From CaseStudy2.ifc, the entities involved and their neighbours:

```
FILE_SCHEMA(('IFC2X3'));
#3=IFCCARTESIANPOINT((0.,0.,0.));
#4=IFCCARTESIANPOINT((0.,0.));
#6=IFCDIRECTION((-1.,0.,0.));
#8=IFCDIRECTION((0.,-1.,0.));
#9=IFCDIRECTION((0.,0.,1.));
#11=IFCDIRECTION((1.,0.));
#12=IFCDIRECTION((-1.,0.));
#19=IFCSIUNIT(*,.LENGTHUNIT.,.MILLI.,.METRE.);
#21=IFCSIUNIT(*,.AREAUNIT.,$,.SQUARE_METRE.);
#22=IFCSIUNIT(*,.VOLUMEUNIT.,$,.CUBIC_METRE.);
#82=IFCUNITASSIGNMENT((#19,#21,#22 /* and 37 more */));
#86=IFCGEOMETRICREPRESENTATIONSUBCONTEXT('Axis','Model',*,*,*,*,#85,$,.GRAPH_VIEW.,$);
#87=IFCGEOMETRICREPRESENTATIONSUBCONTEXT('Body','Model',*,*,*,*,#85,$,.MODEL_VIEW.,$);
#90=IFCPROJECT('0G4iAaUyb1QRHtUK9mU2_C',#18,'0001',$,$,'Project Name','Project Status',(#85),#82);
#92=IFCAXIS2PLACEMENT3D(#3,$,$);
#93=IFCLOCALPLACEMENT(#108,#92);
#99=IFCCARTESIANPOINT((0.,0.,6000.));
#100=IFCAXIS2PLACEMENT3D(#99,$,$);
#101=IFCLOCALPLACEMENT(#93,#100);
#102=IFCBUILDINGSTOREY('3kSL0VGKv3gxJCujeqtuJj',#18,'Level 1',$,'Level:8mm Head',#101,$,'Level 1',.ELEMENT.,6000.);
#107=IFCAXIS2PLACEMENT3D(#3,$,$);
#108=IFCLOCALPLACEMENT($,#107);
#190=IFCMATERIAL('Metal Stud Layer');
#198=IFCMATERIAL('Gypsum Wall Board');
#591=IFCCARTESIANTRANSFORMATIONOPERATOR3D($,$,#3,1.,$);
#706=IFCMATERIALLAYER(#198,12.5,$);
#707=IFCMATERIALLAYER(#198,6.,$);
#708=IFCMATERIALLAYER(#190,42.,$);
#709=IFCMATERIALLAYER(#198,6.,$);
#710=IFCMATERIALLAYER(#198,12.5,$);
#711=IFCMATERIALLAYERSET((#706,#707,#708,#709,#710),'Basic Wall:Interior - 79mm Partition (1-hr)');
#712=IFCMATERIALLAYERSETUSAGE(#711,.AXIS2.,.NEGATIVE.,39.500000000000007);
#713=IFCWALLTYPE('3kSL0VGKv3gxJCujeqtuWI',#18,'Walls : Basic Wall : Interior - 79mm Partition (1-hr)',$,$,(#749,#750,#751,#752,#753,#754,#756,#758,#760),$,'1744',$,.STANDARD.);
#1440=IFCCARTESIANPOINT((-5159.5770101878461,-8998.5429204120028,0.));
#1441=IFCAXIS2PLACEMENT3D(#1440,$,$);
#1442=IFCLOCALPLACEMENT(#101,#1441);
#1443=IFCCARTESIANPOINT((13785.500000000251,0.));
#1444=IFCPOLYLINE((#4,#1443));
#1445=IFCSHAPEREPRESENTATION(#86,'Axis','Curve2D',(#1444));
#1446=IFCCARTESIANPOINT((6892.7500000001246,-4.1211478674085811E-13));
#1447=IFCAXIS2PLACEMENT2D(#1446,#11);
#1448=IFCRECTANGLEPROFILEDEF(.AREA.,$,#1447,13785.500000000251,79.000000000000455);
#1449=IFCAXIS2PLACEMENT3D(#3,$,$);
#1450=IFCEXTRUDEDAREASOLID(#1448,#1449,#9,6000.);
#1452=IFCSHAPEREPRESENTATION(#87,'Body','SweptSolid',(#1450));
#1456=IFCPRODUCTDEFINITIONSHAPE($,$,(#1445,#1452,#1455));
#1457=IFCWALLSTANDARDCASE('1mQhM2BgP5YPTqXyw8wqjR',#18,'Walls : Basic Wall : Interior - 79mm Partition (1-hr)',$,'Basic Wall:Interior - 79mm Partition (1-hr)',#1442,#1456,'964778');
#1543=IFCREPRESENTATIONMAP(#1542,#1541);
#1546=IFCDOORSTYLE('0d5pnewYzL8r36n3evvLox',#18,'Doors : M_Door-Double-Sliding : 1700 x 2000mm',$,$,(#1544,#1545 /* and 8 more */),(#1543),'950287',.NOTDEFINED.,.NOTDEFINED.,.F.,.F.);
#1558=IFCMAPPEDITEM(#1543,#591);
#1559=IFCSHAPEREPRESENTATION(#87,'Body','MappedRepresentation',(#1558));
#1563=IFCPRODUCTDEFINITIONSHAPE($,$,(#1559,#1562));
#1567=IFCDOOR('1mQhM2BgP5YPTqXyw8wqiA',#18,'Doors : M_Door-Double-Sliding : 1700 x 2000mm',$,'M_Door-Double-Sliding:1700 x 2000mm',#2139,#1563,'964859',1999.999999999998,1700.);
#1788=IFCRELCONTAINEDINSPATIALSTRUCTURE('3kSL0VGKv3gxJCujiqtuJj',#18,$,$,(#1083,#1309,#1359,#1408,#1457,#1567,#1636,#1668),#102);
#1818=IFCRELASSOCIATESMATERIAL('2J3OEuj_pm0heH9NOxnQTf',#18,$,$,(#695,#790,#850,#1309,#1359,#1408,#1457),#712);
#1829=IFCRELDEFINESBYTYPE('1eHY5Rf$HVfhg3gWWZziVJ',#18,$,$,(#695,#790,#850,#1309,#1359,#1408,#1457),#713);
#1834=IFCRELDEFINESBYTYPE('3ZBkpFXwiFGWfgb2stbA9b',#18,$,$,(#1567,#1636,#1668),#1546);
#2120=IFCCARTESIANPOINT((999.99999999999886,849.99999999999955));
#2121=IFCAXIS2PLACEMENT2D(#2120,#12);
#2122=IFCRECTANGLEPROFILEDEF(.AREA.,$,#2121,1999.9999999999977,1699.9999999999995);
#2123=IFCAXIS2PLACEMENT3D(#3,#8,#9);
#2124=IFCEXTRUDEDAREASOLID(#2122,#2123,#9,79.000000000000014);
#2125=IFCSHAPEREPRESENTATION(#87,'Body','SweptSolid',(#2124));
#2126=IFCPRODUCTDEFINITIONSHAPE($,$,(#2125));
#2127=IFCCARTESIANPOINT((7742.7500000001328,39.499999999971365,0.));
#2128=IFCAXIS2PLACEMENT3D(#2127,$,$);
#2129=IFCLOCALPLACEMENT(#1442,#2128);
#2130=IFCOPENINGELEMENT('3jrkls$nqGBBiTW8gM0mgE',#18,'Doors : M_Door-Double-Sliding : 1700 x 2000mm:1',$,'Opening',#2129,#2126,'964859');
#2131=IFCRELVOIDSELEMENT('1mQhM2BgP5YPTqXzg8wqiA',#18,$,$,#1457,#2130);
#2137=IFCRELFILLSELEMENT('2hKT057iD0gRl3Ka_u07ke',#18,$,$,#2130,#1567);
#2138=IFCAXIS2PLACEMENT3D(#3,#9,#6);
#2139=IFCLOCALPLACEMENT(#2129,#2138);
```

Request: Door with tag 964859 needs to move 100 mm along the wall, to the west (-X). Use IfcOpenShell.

```python
import ifcopenshell
import ifcopenshell.api.geometry
import ifcopenshell.util.placement

model = ifcopenshell.open("CaseStudy2.ifc")

door = model.by_guid("1mQhM2BgP5YPTqXyw8wqiA")
opening = door.FillsVoids[0].RelatingOpeningElement
wall = opening.VoidsElements[0].RelatingBuildingElement

wall_matrix = ifcopenshell.util.placement.get_local_placement(wall.ObjectPlacement)
shift = wall_matrix[:3, 0] * -100.0
before = ifcopenshell.util.placement.get_local_placement(door.ObjectPlacement)[:3, 3].copy()

# The door is placed relative to its opening, so it follows when the opening moves.
matrix = ifcopenshell.util.placement.get_local_placement(opening.ObjectPlacement)
matrix[:3, 3] += shift
ifcopenshell.api.geometry.edit_object_placement(
    model, product=opening, matrix=matrix, is_si=False, should_transform_children=True
)

after = ifcopenshell.util.placement.get_local_placement(door.ObjectPlacement)[:3, 3]
print("door moved by", (after - before).round(3) + 0.0)

model.write("CaseStudy2_rev.ifc")
```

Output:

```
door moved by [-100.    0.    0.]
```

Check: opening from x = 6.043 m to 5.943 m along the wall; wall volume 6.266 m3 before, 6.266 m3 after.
